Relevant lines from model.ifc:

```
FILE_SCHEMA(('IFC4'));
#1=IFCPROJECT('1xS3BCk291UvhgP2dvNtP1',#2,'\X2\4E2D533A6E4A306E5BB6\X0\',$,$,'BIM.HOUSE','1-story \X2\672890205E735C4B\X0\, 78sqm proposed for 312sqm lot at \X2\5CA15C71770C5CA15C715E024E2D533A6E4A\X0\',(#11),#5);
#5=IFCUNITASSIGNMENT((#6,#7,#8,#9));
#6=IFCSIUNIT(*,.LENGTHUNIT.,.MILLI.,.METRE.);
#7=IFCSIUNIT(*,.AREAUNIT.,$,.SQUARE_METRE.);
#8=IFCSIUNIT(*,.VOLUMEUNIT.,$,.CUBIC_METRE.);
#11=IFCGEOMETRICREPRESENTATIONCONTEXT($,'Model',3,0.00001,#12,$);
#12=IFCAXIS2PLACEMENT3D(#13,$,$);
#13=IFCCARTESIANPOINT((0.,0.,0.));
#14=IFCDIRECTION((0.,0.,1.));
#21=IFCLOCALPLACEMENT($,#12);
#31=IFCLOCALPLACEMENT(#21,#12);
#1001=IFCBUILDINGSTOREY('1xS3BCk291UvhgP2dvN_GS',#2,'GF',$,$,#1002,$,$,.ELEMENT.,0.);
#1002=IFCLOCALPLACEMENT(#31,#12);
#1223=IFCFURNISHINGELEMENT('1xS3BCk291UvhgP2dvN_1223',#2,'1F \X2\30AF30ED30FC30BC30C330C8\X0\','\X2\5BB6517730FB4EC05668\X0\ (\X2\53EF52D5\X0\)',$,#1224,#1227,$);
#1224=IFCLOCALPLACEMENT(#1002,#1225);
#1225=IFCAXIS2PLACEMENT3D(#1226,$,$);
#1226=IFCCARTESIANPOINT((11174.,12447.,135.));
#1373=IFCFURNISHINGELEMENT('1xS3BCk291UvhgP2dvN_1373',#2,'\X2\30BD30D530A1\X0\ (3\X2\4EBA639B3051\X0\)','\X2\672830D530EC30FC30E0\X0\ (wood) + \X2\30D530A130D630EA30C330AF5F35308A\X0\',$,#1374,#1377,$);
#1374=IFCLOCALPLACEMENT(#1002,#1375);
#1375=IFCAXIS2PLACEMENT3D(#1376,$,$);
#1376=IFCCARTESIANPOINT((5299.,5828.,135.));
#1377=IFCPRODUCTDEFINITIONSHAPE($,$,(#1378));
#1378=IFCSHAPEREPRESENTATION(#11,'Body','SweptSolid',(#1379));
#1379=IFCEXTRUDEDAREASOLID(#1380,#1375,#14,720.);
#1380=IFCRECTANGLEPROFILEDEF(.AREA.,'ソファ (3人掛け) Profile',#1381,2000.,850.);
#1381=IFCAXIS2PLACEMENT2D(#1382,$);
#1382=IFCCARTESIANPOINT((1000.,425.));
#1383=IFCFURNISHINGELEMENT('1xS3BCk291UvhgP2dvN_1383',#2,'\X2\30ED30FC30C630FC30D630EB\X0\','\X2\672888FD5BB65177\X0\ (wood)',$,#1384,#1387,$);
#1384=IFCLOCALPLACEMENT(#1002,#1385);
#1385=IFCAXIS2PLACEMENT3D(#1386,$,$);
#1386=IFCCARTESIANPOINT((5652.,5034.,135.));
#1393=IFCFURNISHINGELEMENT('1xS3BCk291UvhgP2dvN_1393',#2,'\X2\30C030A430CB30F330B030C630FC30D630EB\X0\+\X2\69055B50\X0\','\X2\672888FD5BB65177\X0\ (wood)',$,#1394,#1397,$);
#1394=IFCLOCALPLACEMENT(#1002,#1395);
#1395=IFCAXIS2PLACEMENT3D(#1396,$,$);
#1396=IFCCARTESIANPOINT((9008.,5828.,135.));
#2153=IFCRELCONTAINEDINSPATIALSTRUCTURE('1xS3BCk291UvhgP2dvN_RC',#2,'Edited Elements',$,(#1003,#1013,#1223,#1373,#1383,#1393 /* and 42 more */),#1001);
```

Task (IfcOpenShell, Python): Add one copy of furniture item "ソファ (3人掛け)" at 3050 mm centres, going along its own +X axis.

```python
import ifcopenshell
import ifcopenshell.api.geometry
import ifcopenshell.api.root
import ifcopenshell.util.element
import ifcopenshell.util.placement

model = ifcopenshell.open("model.ifc")


def reuse_history(source, copy):
    """copy_class also copies each property set's owner history, people and application; keep the originals."""
    for rel in copy.IsDefinedBy:
        if rel.is_a("IfcRelDefinesByProperties") and (history := rel.RelatingPropertyDefinition.OwnerHistory):
            rel.RelatingPropertyDefinition.OwnerHistory = source.OwnerHistory
            ifcopenshell.util.element.remove_deep2(model, history)


source = model.by_guid("1xS3BCk291UvhgP2dvN_1373")
base = ifcopenshell.util.placement.get_local_placement(source.ObjectPlacement)
step = base[:3, 0] * 3050.0

for i in range(1, 2):
    copy = ifcopenshell.api.root.copy_class(model, product=source)
    copy.Representation = ifcopenshell.util.element.copy_deep(
        model, source.Representation, exclude=["IfcGeometricRepresentationContext", "IfcRepresentationMap"]
    )
    reuse_history(source, copy)
    matrix = base.copy()
    matrix[:3, 3] += i * step
    print("added at", matrix[:3, 3].round(3) + 0.0)
    ifcopenshell.api.geometry.edit_object_placement(model, product=copy, matrix=matrix, is_si=False)

model.write("model_v2.ifc")
```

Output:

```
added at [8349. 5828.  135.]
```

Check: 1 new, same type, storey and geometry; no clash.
